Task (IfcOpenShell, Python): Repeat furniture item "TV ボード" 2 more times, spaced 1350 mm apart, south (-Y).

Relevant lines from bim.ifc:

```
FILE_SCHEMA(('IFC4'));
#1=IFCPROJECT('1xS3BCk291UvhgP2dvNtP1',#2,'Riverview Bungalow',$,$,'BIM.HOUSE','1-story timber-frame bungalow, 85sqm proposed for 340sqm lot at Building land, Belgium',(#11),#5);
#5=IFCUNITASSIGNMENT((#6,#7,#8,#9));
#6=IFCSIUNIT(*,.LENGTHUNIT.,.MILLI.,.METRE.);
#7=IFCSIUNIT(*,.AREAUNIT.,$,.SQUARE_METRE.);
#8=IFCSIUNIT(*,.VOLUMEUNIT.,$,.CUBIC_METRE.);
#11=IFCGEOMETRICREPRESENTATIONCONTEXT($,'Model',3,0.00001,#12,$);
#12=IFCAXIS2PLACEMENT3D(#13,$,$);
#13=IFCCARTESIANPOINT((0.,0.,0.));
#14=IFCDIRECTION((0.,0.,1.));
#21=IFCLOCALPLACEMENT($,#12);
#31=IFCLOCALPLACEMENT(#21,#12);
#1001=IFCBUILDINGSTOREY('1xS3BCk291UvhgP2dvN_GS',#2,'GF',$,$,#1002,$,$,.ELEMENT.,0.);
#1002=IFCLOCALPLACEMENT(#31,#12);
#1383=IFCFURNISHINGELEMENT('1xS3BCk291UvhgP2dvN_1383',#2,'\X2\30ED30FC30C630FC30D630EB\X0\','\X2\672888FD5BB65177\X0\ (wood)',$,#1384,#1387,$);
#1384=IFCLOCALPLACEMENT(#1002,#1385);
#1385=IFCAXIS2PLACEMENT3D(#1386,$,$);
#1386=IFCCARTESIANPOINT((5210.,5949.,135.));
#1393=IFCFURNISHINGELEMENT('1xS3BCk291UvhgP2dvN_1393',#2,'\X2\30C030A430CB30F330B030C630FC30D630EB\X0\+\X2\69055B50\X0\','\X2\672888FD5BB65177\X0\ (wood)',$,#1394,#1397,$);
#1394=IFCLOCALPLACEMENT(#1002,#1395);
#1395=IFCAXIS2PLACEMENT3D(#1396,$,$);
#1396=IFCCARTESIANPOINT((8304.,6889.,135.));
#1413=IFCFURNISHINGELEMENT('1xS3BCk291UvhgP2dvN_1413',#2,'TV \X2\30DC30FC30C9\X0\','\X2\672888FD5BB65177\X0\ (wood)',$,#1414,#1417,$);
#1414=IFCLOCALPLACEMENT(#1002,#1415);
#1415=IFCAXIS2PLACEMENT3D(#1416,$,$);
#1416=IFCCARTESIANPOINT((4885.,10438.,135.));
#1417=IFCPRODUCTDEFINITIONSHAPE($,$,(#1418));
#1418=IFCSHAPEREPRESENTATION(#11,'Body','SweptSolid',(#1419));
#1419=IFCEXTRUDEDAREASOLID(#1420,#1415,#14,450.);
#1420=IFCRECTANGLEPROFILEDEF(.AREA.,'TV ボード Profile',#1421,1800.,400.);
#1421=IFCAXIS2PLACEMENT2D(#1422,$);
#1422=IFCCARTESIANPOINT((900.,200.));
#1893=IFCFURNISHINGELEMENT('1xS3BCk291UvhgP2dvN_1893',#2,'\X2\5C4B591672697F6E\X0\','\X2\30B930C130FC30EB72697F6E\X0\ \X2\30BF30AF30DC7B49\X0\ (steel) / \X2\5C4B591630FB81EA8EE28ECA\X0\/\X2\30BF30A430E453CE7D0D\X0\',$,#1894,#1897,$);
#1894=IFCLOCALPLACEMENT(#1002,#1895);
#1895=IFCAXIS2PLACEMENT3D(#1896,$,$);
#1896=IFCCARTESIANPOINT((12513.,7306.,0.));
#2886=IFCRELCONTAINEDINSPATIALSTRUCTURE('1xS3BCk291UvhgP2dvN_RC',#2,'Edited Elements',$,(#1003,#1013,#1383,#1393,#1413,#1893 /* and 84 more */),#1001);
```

```python
import numpy as np
import ifcopenshell
import ifcopenshell.api.geometry
import ifcopenshell.api.root
import ifcopenshell.util.element
import ifcopenshell.util.placement
import ifcopenshell.util.unit

model = ifcopenshell.open("bim.ifc")
unit_scale = ifcopenshell.util.unit.calculate_unit_scale(model)


def reuse_history(source, copy):
    """copy_class also copies each property set's owner history, people and application; keep the originals."""
    for rel in copy.IsDefinedBy:
        if rel.is_a("IfcRelDefinesByProperties") and (history := rel.RelatingPropertyDefinition.OwnerHistory):
            rel.RelatingPropertyDefinition.OwnerHistory = source.OwnerHistory
            ifcopenshell.util.element.remove_deep2(model, history)


source = model.by_id(1413)
base = ifcopenshell.util.placement.get_local_placement(source.ObjectPlacement)
step = np.array([0.0, -1.0, 0.0]) * 1.35 / unit_scale

for i in range(1, 3):
    copy = ifcopenshell.api.root.copy_class(model, product=source)
    copy.Representation = ifcopenshell.util.element.copy_deep(
        model, source.Representation, exclude=["IfcGeometricRepresentationContext", "IfcRepresentationMap"]
    )
    reuse_history(source, copy)
    matrix = base.copy()
    matrix[:3, 3] += i * step
    print("added at", matrix[:3, 3].round(3) + 0.0)
    ifcopenshell.api.geometry.edit_object_placement(model, product=copy, matrix=matrix, is_si=False)

model.write("bim_updated.ifc")
```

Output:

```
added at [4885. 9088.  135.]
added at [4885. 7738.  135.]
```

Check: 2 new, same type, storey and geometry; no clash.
